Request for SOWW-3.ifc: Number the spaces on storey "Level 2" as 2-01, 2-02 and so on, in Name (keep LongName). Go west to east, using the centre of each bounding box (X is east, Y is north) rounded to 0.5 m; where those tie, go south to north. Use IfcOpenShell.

First a look at what the model holds.

```python
import ifcopenshell
import ifcopenshell.util.element
import ifcopenshell.util.placement

model = ifcopenshell.open("SOWW-3.ifc")
print(model.schema)
storey = next(s for s in model.by_type("IfcBuildingStorey") if s.Name == "Level 2")
spaces = [e for e in ifcopenshell.util.element.get_decomposition(storey) if e.is_a("IfcSpace")]
for e in sorted(spaces, key=lambda e: e.id()):
    origin = ifcopenshell.util.placement.get_local_placement(e.ObjectPlacement)[:3, 3]
    print(e.id(), e.Name, e.LongName, origin.round(2) + 0.0, sep=" | ")
```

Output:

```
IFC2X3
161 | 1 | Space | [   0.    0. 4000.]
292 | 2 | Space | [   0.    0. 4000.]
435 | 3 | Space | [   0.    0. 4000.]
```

```python
import ifcopenshell
import ifcopenshell.geom
import ifcopenshell.util.element
import ifcopenshell.util.shape

model = ifcopenshell.open("SOWW-3.ifc")
settings = ifcopenshell.geom.settings()
settings.set("use-world-coords", True)


def centre(element):
    shape = ifcopenshell.geom.create_shape(settings, element)
    return ifcopenshell.util.shape.get_bbox_centroid(shape.geometry)


storey = next(s for s in model.by_type("IfcBuildingStorey") if s.Name == "Level 2")
spaces = [e for e in ifcopenshell.util.element.get_decomposition(storey) if e.is_a("IfcSpace")]

# Insertion points can sit at a corner or the storey origin, so sort by the geometry (in metres).
centres = {e: centre(e) for e in spaces}
spaces.sort(key=lambda e: (round(centres[e][0] / 0.5), centres[e][1]))

for i, e in enumerate(spaces, start=1):
    number = f"2-{i:02d}"
    e.Name = number
    print(e.id(), number)

model.write("SOWW-3_edited.ifc")
```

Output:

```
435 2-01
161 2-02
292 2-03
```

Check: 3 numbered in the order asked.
